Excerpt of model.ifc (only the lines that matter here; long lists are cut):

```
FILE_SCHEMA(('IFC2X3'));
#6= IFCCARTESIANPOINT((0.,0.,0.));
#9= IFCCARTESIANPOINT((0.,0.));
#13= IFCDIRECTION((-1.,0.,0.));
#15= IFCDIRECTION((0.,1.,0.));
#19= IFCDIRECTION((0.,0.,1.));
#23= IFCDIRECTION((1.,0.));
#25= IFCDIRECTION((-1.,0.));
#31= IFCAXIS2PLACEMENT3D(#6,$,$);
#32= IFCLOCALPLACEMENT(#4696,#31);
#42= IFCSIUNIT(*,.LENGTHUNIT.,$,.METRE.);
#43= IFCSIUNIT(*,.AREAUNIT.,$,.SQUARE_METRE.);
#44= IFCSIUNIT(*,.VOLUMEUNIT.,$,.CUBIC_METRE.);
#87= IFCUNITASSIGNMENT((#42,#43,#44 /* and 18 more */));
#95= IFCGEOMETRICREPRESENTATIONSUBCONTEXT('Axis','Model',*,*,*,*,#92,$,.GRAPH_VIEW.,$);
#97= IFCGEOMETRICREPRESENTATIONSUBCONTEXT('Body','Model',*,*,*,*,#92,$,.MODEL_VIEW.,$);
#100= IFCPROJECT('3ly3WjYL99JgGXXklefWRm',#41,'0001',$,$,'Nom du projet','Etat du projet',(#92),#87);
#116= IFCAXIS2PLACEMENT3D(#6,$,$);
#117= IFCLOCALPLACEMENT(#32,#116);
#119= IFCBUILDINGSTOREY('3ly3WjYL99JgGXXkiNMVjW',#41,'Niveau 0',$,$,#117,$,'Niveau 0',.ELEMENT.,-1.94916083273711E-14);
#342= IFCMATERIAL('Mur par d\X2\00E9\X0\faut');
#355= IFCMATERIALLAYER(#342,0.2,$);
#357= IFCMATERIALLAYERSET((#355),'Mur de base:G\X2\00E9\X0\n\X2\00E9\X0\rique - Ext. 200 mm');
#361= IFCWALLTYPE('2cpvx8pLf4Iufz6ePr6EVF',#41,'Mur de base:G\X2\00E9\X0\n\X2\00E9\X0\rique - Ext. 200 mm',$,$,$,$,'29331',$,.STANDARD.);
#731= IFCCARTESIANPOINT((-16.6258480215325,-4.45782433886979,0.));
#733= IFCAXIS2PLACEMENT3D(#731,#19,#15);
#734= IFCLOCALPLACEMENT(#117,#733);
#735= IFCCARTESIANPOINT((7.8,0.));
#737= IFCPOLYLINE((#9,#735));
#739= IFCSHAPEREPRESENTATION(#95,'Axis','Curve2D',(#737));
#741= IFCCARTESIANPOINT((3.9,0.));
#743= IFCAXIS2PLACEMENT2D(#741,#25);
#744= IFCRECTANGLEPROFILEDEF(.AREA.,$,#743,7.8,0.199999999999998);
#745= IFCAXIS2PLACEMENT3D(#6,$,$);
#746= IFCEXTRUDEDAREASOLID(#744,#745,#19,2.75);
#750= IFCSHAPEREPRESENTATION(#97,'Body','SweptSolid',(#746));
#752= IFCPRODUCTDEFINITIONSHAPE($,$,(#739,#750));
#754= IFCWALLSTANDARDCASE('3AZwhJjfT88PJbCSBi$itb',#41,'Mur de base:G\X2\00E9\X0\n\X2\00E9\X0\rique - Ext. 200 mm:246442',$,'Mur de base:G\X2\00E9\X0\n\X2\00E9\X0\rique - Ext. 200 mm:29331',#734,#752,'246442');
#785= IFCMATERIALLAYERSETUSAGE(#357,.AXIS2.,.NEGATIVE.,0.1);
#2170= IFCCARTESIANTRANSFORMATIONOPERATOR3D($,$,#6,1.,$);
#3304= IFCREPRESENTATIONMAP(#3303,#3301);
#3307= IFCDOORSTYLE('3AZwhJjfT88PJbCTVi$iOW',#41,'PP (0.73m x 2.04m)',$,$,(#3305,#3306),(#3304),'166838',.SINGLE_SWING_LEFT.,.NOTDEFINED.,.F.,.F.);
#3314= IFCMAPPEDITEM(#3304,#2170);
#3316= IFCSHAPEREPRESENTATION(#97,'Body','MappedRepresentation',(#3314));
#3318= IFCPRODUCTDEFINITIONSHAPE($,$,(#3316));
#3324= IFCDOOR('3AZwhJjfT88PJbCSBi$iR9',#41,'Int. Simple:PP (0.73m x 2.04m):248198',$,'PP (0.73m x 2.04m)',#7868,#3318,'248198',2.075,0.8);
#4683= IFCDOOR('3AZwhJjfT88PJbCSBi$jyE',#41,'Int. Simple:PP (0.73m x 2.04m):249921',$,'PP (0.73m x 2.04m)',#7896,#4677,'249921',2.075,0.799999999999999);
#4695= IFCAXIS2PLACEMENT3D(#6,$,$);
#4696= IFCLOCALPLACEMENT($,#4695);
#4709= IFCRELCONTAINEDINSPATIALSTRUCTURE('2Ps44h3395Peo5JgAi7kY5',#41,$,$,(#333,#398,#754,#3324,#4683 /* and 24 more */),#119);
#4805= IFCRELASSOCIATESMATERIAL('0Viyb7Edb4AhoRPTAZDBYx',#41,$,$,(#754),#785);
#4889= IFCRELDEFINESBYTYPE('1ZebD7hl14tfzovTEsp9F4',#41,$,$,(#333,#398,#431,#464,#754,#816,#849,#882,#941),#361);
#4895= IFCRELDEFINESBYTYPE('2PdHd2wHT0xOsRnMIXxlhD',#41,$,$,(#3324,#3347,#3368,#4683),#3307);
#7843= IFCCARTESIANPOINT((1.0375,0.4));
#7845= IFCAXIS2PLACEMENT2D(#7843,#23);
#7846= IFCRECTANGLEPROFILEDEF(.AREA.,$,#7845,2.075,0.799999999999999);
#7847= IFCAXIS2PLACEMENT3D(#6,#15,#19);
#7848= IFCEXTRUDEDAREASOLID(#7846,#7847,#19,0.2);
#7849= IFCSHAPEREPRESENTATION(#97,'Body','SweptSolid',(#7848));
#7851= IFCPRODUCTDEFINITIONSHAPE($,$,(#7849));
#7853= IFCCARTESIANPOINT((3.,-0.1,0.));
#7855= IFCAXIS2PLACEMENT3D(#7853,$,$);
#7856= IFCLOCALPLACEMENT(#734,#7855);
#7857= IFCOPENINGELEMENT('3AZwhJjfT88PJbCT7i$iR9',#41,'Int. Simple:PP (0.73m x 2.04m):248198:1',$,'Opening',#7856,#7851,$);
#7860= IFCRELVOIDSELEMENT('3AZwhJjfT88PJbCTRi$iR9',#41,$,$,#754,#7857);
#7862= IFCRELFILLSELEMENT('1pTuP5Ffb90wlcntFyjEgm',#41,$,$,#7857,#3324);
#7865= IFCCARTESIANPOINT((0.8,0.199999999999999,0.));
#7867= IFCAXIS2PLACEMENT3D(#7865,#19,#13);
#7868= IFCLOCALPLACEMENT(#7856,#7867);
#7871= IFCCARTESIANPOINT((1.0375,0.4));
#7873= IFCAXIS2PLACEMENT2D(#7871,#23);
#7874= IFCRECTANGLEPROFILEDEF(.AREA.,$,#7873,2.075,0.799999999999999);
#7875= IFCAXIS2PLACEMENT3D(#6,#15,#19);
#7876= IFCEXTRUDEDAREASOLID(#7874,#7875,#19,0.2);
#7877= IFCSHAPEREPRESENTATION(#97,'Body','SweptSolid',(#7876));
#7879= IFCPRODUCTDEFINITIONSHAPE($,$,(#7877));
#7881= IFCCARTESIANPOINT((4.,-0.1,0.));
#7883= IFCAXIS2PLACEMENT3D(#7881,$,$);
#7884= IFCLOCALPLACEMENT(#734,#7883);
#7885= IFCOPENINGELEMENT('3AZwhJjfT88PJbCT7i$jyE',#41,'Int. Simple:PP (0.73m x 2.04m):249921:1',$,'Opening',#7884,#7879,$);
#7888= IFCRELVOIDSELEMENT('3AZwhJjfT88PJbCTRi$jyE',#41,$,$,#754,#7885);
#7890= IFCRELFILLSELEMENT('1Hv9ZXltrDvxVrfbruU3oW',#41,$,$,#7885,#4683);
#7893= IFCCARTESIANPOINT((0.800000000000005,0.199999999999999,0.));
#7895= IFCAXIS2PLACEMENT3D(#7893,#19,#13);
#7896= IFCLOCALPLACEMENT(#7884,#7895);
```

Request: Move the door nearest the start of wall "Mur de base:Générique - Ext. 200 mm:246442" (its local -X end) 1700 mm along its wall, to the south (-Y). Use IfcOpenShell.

```python
import ifcopenshell
import ifcopenshell.api.geometry
import ifcopenshell.util.placement

model = ifcopenshell.open("model.ifc")

door = model.by_guid("3AZwhJjfT88PJbCSBi$iR9")
opening = door.FillsVoids[0].RelatingOpeningElement
wall = opening.VoidsElements[0].RelatingBuildingElement

wall_matrix = ifcopenshell.util.placement.get_local_placement(wall.ObjectPlacement)
shift = wall_matrix[:3, 0] * -1.7
before = ifcopenshell.util.placement.get_local_placement(door.ObjectPlacement)[:3, 3].copy()

# The door is placed relative to its opening, so it follows when the opening moves.
matrix = ifcopenshell.util.placement.get_local_placement(opening.ObjectPlacement)
matrix[:3, 3] += shift
ifcopenshell.api.geometry.edit_object_placement(
    model, product=opening, matrix=matrix, is_si=False, should_transform_children=True
)

after = ifcopenshell.util.placement.get_local_placement(door.ObjectPlacement)[:3, 3]
print("door moved by", (after - before).round(3) + 0.0)

model.write("model-out.ifc")
```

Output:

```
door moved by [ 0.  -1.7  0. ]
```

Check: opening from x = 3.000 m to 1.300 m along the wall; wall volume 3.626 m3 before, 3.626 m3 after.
